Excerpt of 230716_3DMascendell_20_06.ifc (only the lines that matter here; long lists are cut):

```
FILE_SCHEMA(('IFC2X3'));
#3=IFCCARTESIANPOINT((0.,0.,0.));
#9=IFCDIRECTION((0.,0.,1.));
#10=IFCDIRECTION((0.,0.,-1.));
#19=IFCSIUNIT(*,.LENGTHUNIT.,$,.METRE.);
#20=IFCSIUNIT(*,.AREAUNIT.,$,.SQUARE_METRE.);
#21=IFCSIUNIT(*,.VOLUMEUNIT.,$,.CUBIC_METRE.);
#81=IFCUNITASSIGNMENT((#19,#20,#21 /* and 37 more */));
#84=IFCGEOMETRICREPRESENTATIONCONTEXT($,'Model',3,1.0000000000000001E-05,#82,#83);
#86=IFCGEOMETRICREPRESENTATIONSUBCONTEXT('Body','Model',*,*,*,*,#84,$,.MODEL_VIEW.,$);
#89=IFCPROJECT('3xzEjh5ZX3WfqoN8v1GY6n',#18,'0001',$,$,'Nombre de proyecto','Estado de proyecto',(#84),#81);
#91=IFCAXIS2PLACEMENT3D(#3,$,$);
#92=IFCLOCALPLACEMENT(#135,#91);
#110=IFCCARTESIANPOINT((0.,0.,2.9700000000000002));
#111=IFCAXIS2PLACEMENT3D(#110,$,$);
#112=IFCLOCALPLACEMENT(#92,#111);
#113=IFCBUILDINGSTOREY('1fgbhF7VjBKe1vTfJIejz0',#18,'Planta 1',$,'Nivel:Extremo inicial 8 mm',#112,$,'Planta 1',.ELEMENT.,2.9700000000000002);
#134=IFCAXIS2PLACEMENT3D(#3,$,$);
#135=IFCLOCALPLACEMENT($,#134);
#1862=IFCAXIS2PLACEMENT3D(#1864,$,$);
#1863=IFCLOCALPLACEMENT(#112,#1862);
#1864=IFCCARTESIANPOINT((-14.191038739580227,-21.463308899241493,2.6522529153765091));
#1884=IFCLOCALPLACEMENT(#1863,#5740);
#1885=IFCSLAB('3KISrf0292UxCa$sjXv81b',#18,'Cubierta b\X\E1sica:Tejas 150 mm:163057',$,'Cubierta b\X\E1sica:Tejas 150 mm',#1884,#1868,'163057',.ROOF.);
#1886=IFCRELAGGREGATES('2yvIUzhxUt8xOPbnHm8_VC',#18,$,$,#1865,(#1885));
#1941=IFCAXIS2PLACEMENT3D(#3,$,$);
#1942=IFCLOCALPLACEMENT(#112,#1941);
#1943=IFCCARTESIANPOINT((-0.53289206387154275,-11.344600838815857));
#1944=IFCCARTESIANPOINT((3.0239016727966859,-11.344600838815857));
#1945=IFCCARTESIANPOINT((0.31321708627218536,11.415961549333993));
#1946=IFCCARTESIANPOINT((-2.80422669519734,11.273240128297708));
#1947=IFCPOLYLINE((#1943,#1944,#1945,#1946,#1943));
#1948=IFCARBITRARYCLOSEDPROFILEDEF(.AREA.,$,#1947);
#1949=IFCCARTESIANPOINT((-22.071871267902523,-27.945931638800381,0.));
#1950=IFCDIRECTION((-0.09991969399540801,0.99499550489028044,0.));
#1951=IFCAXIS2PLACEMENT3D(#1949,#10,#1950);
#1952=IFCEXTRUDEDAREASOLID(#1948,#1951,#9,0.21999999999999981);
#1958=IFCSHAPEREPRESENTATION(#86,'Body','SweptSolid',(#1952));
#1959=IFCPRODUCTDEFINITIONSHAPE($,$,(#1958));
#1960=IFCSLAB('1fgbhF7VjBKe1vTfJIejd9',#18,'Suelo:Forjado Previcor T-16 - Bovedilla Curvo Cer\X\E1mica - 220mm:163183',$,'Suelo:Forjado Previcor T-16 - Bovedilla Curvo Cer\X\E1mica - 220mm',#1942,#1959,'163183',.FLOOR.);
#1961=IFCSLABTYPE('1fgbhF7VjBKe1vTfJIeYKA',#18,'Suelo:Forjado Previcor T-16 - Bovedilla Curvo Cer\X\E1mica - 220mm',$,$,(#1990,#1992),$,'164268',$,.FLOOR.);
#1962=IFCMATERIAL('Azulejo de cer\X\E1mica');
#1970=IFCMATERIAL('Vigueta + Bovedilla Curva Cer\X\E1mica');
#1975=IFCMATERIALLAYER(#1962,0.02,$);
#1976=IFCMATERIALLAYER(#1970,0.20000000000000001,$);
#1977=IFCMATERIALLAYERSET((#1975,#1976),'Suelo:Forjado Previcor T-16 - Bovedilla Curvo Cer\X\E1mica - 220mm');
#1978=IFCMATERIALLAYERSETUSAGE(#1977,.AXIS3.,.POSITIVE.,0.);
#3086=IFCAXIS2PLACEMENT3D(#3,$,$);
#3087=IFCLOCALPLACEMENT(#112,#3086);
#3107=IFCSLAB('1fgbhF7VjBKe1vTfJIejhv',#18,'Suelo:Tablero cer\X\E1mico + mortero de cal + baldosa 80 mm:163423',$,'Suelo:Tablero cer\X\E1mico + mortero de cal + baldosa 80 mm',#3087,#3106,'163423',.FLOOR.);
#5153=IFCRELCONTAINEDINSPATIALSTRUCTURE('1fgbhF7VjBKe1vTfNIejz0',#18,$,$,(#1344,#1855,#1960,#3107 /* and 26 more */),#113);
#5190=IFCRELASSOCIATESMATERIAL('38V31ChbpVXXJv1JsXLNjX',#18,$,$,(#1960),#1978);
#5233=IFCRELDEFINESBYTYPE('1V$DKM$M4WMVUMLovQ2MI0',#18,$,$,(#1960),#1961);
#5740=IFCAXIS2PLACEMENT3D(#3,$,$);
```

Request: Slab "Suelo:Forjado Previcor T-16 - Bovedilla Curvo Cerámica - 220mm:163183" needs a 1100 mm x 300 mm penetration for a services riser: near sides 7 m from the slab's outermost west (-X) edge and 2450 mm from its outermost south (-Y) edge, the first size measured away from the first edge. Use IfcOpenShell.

```python
import numpy as np
import ifcopenshell
import ifcopenshell.api.feature
import ifcopenshell.api.geometry
import ifcopenshell.api.root
import ifcopenshell.geom
import ifcopenshell.util.placement
import ifcopenshell.util.representation
import ifcopenshell.util.shape
import ifcopenshell.util.unit

model = ifcopenshell.open("230716_3DMascendell_20_06.ifc")
unit_scale = ifcopenshell.util.unit.calculate_unit_scale(model)
settings = ifcopenshell.geom.settings()


def volume(element):
    """Net volume in cubic metres, openings subtracted."""
    shape = ifcopenshell.geom.create_shape(settings, element)
    return ifcopenshell.util.shape.get_volume(shape.geometry)


slab = model.by_guid("1fgbhF7VjBKe1vTfJIejd9")
before = volume(slab)

# Extent in the slab's own axes, in metres. The edges named are its -X and -Y sides.
slab_shape = ifcopenshell.geom.create_shape(settings, slab)
vertices = ifcopenshell.util.shape.get_vertices(slab_shape.geometry)
x_min, y_min, bottom = vertices.min(axis=0)
top = vertices[:, 2].max()

opening = ifcopenshell.api.root.create_entity(model, ifc_class="IfcOpeningElement", name="Services riser opening")
context = ifcopenshell.util.representation.get_context(model, "Model", "Body", "MODEL_VIEW")
width, depth = 1.1, 0.3
outline = [(0.0, 0.0), (width, 0.0), (width, depth), (0.0, depth), (0.0, 0.0)]
# Overshoot both faces by 50 mm so the cut is clean.
shape = ifcopenshell.api.geometry.add_slab_representation(
    model, context=context, depth=top - bottom + 0.1, polyline=outline
)
ifcopenshell.api.geometry.assign_representation(model, product=opening, representation=shape)

matrix = ifcopenshell.util.placement.get_local_placement(slab.ObjectPlacement)
matrix[:, 3] = matrix @ np.append(np.array([x_min + 7, y_min + 2.45, bottom - 0.05]) / unit_scale, 1.0)
ifcopenshell.api.geometry.edit_object_placement(model, product=opening, matrix=matrix, is_si=False)
ifcopenshell.api.feature.add_feature(model, feature=opening, element=slab)

after = volume(slab)

print(f"slab volume {before:.3f} -> {after:.3f} m3")

model.write("230716_3DMascendell_20_06_rev.ifc")
```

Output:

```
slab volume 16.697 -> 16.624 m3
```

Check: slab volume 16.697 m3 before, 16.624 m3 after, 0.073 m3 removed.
